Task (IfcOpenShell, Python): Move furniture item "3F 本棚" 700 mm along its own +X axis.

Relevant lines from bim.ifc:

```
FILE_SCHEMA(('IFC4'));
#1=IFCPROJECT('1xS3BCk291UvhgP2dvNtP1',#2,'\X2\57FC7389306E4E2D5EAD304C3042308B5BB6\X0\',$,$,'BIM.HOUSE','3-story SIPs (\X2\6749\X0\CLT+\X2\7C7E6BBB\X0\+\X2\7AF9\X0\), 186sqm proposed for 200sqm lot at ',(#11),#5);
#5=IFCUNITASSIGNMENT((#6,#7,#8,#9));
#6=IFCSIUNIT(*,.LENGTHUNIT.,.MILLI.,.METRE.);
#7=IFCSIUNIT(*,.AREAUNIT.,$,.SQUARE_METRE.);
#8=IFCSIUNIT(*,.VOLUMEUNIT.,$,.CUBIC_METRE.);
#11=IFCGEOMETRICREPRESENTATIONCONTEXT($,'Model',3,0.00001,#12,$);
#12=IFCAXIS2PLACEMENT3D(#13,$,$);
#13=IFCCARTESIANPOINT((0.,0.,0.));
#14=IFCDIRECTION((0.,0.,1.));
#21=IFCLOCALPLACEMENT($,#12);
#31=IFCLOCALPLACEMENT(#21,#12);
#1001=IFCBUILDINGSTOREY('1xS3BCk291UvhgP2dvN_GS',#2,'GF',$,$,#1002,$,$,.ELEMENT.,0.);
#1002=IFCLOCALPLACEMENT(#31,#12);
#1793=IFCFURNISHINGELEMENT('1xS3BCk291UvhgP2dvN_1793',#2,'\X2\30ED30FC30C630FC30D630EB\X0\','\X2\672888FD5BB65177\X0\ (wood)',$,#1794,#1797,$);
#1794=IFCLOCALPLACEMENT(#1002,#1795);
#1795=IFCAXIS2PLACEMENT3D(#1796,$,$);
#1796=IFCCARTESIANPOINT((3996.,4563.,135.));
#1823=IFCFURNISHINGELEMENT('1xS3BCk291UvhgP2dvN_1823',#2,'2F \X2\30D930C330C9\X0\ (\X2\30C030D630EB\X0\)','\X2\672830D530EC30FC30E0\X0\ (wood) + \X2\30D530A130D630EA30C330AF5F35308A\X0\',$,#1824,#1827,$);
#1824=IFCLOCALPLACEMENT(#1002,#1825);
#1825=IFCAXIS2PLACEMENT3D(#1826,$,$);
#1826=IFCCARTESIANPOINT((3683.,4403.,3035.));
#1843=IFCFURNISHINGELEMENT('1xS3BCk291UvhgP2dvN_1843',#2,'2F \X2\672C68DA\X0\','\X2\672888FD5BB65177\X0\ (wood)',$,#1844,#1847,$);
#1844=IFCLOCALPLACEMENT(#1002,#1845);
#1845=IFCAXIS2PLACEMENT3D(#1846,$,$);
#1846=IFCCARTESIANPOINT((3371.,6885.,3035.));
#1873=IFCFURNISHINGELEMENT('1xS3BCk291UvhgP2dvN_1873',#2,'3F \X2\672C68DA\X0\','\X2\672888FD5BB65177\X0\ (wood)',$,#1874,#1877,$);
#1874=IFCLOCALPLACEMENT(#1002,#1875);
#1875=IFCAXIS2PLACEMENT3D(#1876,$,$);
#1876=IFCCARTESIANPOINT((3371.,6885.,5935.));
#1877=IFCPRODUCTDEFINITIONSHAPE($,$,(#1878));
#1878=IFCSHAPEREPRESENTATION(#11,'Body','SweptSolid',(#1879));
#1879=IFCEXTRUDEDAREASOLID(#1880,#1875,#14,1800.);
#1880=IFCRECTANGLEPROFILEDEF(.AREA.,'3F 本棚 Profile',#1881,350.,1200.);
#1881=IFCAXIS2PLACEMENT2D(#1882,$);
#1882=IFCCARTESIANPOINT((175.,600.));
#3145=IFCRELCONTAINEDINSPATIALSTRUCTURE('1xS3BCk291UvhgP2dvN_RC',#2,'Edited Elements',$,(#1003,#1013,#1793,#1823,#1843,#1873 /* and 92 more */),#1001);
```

```python
import ifcopenshell
import ifcopenshell.api.geometry
import ifcopenshell.util.placement

model = ifcopenshell.open("bim.ifc")

item = model.by_guid("1xS3BCk291UvhgP2dvN_1873")
matrix = ifcopenshell.util.placement.get_local_placement(item.ObjectPlacement)
matrix[:3, 3] += matrix[:3, 0] * 700.0
ifcopenshell.api.geometry.edit_object_placement(model, product=item, matrix=matrix, is_si=False)

print(ifcopenshell.util.placement.get_local_placement(item.ObjectPlacement).round(3) + 0.0)

model.write("bim_v2.ifc")
```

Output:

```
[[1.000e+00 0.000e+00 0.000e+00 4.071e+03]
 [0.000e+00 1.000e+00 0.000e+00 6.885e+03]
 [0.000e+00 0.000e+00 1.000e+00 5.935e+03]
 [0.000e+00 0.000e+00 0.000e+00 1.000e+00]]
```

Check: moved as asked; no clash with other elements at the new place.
